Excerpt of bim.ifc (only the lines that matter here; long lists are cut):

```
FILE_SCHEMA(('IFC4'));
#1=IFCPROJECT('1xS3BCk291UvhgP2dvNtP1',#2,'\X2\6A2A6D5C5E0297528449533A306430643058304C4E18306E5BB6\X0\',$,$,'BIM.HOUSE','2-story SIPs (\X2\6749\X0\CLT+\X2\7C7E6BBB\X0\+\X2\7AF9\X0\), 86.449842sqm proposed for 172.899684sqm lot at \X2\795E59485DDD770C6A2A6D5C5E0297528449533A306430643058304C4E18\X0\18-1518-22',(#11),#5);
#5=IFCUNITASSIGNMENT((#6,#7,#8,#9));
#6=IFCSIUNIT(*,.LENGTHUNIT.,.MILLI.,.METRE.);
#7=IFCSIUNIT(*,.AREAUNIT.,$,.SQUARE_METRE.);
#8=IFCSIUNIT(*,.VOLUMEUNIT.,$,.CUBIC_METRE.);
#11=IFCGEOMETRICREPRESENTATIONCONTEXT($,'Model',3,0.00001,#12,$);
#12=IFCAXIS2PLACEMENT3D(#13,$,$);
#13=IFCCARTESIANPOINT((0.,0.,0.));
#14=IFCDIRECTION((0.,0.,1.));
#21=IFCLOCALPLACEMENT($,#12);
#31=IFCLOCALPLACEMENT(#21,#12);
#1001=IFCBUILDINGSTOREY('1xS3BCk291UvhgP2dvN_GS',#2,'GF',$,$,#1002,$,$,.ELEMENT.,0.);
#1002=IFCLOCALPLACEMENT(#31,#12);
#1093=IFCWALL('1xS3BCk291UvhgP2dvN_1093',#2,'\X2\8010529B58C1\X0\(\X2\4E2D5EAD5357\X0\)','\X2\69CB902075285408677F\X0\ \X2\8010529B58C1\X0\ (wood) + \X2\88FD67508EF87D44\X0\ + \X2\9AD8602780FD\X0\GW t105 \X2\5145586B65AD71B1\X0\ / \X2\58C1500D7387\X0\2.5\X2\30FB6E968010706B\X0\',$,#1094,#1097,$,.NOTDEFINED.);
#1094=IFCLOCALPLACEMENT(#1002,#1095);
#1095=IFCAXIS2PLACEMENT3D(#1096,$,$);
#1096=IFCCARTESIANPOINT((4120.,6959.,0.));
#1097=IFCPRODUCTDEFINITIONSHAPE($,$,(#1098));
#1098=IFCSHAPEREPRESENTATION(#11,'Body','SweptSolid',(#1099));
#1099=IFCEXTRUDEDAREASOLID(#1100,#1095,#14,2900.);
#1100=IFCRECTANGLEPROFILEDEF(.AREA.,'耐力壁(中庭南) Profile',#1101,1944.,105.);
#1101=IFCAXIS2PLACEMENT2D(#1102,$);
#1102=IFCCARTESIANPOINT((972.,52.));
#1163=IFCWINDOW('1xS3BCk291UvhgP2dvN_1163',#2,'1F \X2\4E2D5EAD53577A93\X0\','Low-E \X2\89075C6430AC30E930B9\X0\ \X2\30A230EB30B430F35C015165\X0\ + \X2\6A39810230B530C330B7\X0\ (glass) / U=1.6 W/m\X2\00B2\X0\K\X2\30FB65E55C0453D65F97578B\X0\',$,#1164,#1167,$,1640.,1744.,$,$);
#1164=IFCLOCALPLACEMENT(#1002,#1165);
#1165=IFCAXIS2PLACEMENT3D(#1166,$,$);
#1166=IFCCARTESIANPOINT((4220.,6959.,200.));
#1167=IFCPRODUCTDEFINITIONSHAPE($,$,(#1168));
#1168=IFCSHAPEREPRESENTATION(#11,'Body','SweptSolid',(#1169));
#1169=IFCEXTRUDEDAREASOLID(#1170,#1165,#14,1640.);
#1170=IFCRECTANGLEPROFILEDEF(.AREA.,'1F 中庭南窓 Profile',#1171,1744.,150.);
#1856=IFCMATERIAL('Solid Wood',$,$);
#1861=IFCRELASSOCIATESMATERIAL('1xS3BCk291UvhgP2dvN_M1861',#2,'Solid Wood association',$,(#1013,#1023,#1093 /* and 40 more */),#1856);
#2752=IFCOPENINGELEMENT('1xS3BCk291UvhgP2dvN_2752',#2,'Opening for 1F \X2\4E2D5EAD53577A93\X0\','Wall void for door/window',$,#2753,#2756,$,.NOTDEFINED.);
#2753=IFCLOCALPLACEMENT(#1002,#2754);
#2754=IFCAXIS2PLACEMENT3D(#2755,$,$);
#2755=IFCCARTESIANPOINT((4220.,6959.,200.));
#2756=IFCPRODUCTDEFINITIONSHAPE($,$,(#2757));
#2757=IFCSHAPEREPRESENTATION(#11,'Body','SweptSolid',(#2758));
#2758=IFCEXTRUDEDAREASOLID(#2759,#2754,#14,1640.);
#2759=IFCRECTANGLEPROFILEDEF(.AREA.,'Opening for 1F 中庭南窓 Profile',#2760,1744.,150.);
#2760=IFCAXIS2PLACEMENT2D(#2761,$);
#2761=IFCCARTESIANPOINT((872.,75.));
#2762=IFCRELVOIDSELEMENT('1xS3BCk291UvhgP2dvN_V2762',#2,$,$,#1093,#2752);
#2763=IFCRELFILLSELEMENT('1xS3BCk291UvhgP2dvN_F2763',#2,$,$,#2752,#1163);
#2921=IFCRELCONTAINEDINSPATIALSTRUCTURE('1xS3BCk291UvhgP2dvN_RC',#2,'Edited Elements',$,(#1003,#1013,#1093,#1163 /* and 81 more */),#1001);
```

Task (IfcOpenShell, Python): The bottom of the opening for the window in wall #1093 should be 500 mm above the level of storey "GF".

```python
import numpy as np
import ifcopenshell
import ifcopenshell.api.geometry
import ifcopenshell.geom
import ifcopenshell.util.element
import ifcopenshell.util.placement
import ifcopenshell.util.shape
import ifcopenshell.util.unit

model = ifcopenshell.open("bim.ifc")
unit_scale = ifcopenshell.util.unit.calculate_unit_scale(model)

window = model.by_guid("1xS3BCk291UvhgP2dvN_1163")
opening = window.FillsVoids[0].RelatingOpeningElement
storey = ifcopenshell.util.element.get_container(window, ifc_class="IfcBuildingStorey")
level = ifcopenshell.util.placement.get_local_placement(storey.ObjectPlacement)[2, 3]

# The opening's origin need not be at the sill, so measure its lowest point.
shape = ifcopenshell.geom.create_shape(ifcopenshell.geom.settings(), opening)
bottom = ifcopenshell.util.shape.get_shape_bottom_elevation(shape, shape.geometry) / unit_scale
dz = level + 0.5 / unit_scale - bottom

shift = np.array([0.0, 0.0, dz])
# The window is not placed relative to its opening, so move both.
for product in (opening, window):
    matrix = ifcopenshell.util.placement.get_local_placement(product.ObjectPlacement)
    matrix[:3, 3] += shift
    ifcopenshell.api.geometry.edit_object_placement(model, product=product, matrix=matrix, is_si=False)

print(f"moved by {dz * unit_scale:+.3f} m")

model.write("bim_rev.ifc")
```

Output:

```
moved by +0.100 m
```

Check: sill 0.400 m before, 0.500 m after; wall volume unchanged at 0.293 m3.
